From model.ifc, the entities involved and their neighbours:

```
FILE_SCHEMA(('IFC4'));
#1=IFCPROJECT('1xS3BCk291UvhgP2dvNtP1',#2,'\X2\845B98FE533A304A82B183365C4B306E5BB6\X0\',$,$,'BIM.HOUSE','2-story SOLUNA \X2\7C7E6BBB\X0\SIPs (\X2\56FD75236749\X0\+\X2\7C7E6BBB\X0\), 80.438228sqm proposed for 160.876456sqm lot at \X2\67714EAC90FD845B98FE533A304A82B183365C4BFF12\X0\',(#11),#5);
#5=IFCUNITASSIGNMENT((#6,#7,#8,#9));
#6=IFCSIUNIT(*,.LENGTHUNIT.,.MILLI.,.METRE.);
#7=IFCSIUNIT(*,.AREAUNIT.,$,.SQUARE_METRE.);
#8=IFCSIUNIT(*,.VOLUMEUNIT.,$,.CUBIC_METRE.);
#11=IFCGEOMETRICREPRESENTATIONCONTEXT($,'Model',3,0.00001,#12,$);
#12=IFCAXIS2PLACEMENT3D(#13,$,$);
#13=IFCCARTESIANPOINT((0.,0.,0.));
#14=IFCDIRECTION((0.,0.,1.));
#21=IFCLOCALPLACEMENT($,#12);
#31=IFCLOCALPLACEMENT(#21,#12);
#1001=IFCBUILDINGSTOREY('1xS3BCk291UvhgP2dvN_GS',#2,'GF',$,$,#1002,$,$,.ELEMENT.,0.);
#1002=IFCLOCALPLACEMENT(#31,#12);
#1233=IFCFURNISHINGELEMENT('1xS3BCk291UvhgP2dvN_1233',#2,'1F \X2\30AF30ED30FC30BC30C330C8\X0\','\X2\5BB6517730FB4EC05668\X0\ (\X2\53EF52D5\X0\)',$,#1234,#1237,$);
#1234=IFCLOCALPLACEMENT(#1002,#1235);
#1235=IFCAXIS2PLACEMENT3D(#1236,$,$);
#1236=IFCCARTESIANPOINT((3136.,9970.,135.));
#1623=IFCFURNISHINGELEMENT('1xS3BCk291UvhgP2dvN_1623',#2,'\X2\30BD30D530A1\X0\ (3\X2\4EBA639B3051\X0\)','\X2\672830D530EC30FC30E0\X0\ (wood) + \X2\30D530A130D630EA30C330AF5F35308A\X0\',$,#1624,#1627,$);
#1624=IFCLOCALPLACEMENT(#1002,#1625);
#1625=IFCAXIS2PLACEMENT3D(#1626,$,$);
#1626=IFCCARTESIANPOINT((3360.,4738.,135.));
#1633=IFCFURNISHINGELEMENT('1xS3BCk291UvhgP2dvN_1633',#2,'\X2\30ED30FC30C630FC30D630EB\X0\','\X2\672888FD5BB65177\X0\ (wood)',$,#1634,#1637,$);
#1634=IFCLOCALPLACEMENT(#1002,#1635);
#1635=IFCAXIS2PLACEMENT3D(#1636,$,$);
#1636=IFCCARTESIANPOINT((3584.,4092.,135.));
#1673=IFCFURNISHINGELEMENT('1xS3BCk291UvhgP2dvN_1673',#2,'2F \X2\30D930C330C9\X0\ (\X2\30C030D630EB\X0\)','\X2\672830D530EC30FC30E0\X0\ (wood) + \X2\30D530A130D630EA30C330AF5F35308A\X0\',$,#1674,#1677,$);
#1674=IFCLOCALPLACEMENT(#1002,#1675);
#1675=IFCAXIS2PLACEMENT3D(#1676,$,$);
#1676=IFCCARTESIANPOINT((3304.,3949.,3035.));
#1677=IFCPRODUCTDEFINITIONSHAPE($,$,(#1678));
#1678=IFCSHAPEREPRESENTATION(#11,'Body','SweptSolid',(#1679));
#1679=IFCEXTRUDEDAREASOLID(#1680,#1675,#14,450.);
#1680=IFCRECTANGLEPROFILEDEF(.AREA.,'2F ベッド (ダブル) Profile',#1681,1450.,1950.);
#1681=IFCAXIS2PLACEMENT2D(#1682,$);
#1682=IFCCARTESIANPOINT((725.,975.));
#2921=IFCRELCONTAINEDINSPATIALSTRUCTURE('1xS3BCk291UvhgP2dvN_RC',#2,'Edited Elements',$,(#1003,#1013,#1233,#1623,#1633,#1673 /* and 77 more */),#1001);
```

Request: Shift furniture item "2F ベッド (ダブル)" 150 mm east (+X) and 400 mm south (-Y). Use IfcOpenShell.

```python
import ifcopenshell
import ifcopenshell.api.geometry
import ifcopenshell.util.placement
import ifcopenshell.util.unit

model = ifcopenshell.open("model.ifc")
unit_scale = ifcopenshell.util.unit.calculate_unit_scale(model)

item = model.by_id(1673)
matrix = ifcopenshell.util.placement.get_local_placement(item.ObjectPlacement)
matrix[0, 3] += 0.15 / unit_scale
matrix[1, 3] -= 0.4 / unit_scale
ifcopenshell.api.geometry.edit_object_placement(model, product=item, matrix=matrix, is_si=False)

print(ifcopenshell.util.placement.get_local_placement(item.ObjectPlacement).round(3) + 0.0)

model.write("model_v2.ifc")
```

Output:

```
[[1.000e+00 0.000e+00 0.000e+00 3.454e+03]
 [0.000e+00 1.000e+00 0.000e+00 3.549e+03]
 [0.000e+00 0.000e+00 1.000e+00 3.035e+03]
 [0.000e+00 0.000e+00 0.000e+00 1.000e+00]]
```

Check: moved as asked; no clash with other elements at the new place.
